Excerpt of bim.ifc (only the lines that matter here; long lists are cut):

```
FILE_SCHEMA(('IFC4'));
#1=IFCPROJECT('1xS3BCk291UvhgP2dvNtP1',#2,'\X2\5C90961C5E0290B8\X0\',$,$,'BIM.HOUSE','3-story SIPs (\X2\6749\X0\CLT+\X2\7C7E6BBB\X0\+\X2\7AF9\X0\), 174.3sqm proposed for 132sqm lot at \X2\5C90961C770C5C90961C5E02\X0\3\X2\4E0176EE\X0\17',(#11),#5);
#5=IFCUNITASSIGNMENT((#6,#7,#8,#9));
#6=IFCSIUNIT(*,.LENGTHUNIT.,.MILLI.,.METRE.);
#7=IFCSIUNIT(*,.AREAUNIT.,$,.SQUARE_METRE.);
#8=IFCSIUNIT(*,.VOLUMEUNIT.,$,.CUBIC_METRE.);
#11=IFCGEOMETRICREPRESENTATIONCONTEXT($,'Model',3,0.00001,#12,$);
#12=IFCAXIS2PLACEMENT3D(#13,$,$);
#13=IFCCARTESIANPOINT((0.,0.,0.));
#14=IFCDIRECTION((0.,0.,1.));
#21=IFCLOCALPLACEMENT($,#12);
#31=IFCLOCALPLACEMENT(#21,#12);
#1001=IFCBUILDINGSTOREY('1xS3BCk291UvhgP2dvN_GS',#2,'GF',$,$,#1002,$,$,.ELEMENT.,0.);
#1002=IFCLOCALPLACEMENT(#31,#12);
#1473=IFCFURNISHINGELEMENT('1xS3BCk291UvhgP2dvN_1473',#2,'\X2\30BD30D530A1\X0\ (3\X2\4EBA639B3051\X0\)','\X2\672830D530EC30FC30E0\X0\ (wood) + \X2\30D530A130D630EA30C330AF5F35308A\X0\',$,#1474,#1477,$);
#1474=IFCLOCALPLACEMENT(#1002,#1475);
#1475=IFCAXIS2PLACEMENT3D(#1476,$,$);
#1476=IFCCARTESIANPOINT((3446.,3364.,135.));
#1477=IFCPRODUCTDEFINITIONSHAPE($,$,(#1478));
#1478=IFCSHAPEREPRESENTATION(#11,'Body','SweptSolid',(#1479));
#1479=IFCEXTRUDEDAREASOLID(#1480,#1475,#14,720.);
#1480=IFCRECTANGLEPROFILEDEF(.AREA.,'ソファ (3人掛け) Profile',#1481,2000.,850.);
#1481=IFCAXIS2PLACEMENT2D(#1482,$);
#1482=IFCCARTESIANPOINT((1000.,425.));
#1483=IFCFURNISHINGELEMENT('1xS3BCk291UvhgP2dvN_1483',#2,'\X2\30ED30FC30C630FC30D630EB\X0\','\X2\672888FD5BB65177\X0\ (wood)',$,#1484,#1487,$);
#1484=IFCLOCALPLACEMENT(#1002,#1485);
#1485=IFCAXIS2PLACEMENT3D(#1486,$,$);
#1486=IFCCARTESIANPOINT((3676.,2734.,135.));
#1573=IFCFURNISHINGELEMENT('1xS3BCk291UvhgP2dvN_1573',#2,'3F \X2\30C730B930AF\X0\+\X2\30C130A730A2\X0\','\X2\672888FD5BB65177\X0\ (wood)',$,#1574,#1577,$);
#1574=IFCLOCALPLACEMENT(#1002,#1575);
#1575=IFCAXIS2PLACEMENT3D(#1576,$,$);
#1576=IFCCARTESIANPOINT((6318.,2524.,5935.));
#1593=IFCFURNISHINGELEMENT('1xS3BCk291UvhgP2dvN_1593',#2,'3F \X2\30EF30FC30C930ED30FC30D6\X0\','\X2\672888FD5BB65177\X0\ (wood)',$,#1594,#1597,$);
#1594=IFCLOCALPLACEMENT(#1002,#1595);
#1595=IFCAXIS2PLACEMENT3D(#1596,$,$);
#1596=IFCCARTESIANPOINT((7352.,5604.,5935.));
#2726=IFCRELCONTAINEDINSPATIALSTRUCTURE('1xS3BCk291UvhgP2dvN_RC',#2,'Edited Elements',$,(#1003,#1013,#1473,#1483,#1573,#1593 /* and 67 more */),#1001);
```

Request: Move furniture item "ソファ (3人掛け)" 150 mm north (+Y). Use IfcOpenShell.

```python
import ifcopenshell
import ifcopenshell.api.geometry
import ifcopenshell.util.placement
import ifcopenshell.util.unit

model = ifcopenshell.open("bim.ifc")
unit_scale = ifcopenshell.util.unit.calculate_unit_scale(model)

item = model.by_guid("1xS3BCk291UvhgP2dvN_1473")
matrix = ifcopenshell.util.placement.get_local_placement(item.ObjectPlacement)
matrix[1, 3] += 0.15 / unit_scale
ifcopenshell.api.geometry.edit_object_placement(model, product=item, matrix=matrix, is_si=False)

print(ifcopenshell.util.placement.get_local_placement(item.ObjectPlacement).round(3) + 0.0)

model.write("bim_v2.ifc")
```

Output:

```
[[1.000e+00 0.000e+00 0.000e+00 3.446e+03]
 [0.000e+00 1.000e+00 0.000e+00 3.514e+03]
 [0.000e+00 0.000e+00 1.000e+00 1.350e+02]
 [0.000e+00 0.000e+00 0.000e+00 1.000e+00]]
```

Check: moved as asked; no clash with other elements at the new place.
